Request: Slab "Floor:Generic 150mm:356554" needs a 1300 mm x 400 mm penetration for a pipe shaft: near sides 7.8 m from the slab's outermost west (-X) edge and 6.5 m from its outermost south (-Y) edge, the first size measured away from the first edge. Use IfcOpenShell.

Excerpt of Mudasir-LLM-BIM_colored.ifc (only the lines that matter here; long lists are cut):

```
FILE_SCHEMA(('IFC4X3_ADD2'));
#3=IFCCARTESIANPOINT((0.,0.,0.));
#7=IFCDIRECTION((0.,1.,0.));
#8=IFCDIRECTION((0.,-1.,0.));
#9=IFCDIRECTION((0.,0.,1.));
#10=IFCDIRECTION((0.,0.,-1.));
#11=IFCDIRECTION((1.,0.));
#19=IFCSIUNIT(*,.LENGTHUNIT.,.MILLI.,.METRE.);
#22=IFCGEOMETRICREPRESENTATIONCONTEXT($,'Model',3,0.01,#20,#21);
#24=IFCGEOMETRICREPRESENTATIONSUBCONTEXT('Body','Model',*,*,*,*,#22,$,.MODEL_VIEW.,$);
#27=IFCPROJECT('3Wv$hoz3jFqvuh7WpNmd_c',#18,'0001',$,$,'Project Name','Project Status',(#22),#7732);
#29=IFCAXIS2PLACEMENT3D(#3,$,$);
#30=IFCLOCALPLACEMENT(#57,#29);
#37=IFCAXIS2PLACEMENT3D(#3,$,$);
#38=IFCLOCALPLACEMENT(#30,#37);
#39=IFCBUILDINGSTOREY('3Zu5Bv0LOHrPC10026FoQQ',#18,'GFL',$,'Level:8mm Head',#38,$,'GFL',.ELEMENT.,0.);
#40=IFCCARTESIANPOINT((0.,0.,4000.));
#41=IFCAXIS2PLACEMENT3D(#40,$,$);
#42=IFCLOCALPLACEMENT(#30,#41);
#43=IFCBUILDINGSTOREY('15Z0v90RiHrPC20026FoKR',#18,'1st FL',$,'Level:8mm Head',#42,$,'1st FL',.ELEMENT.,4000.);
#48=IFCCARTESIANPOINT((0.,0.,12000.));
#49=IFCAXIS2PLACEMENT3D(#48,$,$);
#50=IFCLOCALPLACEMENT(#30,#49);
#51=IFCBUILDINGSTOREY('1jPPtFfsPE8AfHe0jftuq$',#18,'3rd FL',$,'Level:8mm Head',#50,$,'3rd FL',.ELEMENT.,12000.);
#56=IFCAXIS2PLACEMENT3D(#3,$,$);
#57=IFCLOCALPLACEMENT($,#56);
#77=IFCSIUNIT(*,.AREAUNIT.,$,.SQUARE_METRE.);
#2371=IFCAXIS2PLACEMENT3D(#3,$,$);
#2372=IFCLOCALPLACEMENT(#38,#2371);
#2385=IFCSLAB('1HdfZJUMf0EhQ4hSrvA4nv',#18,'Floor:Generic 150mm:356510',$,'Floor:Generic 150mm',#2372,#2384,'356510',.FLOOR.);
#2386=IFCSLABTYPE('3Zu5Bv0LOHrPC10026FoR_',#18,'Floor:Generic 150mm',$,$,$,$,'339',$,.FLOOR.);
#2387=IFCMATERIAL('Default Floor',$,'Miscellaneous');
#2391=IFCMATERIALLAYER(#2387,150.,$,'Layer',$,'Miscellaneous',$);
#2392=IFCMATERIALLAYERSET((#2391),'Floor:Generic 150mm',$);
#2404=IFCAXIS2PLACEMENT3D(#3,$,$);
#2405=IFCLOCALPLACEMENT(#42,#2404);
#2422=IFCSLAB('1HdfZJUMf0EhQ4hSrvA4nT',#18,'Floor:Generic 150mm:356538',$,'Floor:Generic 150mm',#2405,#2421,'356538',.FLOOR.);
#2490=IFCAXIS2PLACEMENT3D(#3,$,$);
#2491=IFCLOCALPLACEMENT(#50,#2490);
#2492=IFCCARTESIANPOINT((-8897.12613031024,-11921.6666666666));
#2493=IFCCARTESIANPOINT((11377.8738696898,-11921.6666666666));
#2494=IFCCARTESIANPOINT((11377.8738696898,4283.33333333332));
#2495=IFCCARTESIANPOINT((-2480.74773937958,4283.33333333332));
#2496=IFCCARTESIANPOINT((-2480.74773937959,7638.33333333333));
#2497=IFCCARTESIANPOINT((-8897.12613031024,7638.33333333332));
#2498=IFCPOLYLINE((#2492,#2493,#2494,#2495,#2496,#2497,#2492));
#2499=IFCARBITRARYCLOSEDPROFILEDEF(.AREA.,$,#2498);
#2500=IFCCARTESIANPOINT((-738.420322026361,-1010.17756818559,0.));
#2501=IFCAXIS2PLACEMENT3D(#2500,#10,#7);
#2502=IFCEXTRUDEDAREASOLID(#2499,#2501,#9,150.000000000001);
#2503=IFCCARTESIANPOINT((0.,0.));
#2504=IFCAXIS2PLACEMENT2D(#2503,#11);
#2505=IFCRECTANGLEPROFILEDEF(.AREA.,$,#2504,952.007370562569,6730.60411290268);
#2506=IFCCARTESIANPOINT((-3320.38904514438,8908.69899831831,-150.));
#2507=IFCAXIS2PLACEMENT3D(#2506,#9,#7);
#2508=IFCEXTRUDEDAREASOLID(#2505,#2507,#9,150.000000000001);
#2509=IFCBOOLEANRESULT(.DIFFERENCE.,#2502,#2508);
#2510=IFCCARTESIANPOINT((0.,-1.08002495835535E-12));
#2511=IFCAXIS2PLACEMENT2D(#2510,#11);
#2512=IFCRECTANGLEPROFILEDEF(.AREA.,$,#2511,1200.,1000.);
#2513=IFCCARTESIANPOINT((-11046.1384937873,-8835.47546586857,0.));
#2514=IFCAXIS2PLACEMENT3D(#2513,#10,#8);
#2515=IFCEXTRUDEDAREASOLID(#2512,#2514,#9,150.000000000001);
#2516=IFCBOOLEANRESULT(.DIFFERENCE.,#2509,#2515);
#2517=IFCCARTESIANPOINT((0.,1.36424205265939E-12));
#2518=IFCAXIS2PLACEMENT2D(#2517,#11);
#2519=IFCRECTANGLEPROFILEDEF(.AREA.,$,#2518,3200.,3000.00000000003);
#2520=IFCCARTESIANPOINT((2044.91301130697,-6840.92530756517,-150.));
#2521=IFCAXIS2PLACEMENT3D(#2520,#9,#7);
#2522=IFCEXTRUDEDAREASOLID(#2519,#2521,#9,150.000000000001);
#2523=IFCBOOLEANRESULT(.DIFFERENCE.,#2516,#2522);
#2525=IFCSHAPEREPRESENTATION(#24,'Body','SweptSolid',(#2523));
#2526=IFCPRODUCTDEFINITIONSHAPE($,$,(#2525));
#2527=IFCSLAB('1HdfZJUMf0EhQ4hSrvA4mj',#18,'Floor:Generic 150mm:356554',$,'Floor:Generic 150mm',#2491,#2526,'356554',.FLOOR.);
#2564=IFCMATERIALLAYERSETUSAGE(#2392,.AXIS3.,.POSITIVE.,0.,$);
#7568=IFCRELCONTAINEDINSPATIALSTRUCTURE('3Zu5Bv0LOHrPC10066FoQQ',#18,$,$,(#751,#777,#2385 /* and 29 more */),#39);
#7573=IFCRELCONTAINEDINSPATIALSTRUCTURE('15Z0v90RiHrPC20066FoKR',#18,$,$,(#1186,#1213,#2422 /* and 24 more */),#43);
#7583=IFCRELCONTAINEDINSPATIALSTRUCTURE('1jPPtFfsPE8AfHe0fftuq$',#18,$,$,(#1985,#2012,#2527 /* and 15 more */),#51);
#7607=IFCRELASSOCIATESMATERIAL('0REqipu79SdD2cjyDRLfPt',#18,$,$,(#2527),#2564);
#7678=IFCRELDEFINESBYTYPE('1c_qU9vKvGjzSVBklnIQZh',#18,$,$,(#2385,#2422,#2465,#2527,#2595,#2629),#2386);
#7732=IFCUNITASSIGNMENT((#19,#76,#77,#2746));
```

```python
import numpy as np
import ifcopenshell
import ifcopenshell.api.feature
import ifcopenshell.api.geometry
import ifcopenshell.api.root
import ifcopenshell.geom
import ifcopenshell.util.placement
import ifcopenshell.util.representation
import ifcopenshell.util.shape
import ifcopenshell.util.unit

model = ifcopenshell.open("Mudasir-LLM-BIM_colored.ifc")
unit_scale = ifcopenshell.util.unit.calculate_unit_scale(model)
settings = ifcopenshell.geom.settings()


def volume(element):
    """Net volume in cubic metres, openings subtracted."""
    shape = ifcopenshell.geom.create_shape(settings, element)
    return ifcopenshell.util.shape.get_volume(shape.geometry)


slab = model.by_guid("1HdfZJUMf0EhQ4hSrvA4mj")
before = volume(slab)

# Extent in the slab's own axes, in metres. The edges named are its -X and -Y sides.
slab_shape = ifcopenshell.geom.create_shape(settings, slab)
vertices = ifcopenshell.util.shape.get_vertices(slab_shape.geometry)
x_min, y_min, bottom = vertices.min(axis=0)
top = vertices[:, 2].max()

opening = ifcopenshell.api.root.create_entity(model, ifc_class="IfcOpeningElement", name="Pipe shaft opening", predefined_type="OPENING")
context = ifcopenshell.util.representation.get_context(model, "Model", "Body", "MODEL_VIEW")
width, depth = 1.3, 0.4
outline = [(0.0, 0.0), (width, 0.0), (width, depth), (0.0, depth), (0.0, 0.0)]
# Overshoot both faces by 50 mm so the cut is clean.
shape = ifcopenshell.api.geometry.add_slab_representation(
    model, context=context, depth=top - bottom + 0.1, polyline=outline
)
ifcopenshell.api.geometry.assign_representation(model, product=opening, representation=shape)

matrix = ifcopenshell.util.placement.get_local_placement(slab.ObjectPlacement)
matrix[:, 3] = matrix @ np.append(np.array([x_min + 7.8, y_min + 6.5, bottom - 0.05]) / unit_scale, 1.0)
ifcopenshell.api.geometry.edit_object_placement(model, product=opening, matrix=matrix, is_si=False)
ifcopenshell.api.feature.add_feature(model, feature=opening, element=slab)

after = volume(slab)

print(f"slab volume {before:.3f} -> {after:.3f} m3")

model.write("Mudasir-LLM-BIM_colored-out.ifc")
```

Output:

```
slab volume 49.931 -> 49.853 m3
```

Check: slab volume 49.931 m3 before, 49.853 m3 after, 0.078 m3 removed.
